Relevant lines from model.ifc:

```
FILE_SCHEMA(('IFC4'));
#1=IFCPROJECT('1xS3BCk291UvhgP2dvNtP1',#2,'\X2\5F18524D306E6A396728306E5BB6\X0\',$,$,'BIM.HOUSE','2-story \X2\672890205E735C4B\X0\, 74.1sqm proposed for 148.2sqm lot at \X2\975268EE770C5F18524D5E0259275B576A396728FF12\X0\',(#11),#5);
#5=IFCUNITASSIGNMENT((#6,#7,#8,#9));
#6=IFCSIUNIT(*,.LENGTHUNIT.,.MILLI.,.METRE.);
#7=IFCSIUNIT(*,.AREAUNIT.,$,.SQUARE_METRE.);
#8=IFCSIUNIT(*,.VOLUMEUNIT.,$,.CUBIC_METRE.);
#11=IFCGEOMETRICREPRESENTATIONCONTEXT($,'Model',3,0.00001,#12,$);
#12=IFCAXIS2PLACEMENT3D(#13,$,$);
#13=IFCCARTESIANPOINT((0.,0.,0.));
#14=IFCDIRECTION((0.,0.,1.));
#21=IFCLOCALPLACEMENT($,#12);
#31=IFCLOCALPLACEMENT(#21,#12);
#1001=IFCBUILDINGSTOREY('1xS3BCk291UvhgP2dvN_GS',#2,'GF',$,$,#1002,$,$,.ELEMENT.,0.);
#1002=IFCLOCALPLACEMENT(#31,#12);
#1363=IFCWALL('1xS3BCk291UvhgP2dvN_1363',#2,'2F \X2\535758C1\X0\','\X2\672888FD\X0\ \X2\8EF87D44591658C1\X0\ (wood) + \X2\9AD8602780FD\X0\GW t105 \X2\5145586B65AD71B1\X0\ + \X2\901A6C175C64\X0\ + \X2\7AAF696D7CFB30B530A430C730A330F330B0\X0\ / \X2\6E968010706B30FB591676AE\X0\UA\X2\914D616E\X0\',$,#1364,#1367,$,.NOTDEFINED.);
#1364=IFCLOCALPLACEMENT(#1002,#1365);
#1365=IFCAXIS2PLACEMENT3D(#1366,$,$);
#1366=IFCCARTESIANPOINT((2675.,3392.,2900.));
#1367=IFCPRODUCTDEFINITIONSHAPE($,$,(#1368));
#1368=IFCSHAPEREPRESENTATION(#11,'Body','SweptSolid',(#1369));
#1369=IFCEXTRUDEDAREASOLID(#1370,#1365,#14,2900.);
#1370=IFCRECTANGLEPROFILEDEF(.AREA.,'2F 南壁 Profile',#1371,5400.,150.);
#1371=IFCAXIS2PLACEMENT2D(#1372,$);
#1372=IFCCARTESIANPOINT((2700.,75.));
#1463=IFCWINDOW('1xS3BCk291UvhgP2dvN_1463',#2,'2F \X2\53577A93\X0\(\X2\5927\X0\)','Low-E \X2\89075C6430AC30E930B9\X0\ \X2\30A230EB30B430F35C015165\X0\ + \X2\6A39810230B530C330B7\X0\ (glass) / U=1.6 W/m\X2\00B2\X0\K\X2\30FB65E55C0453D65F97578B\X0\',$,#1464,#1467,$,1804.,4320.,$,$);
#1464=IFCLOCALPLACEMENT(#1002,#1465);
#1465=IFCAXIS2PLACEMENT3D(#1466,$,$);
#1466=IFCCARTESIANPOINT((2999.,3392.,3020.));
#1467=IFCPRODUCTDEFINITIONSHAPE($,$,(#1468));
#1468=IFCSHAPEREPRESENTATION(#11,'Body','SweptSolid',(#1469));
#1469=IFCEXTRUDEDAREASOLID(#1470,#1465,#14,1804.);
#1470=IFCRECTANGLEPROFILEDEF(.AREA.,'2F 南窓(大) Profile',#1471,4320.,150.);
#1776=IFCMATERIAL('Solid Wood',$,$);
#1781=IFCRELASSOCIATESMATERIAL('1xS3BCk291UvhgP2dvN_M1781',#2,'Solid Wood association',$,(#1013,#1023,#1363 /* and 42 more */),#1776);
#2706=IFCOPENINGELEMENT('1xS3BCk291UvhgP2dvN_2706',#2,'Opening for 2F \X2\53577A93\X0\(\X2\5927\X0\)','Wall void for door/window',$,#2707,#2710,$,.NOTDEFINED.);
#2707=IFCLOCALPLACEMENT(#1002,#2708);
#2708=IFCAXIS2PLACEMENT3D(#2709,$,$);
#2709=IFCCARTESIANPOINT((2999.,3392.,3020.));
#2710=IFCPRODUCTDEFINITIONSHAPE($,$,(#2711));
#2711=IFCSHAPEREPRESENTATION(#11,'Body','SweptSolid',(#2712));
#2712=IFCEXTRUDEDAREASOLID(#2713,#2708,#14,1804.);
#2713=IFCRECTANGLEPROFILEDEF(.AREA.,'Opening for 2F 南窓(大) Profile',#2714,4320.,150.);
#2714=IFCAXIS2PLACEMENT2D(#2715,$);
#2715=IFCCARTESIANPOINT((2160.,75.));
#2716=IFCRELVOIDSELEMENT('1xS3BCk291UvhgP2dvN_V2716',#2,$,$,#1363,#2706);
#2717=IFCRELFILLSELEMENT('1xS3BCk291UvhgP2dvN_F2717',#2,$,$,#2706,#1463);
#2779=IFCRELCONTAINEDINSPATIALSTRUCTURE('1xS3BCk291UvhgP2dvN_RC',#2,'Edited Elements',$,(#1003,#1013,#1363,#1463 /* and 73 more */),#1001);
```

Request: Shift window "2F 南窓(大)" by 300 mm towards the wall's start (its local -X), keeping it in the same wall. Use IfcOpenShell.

```python
import ifcopenshell
import ifcopenshell.api.geometry
import ifcopenshell.util.placement

model = ifcopenshell.open("model.ifc")

window = model.by_id(1463)
opening = window.FillsVoids[0].RelatingOpeningElement
wall = opening.VoidsElements[0].RelatingBuildingElement

wall_matrix = ifcopenshell.util.placement.get_local_placement(wall.ObjectPlacement)
shift = wall_matrix[:3, 0] * -300.0
before = ifcopenshell.util.placement.get_local_placement(window.ObjectPlacement)[:3, 3].copy()

# The window is not placed relative to its opening, so move both.
for product in (opening, window):
    matrix = ifcopenshell.util.placement.get_local_placement(product.ObjectPlacement)
    matrix[:3, 3] += shift
    ifcopenshell.api.geometry.edit_object_placement(model, product=product, matrix=matrix, is_si=False)

after = ifcopenshell.util.placement.get_local_placement(window.ObjectPlacement)[:3, 3]
print("window moved by", (after - before).round(3) + 0.0)

model.write("model_v2.ifc")
```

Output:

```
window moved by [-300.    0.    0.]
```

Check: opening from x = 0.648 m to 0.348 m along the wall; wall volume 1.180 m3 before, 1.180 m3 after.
